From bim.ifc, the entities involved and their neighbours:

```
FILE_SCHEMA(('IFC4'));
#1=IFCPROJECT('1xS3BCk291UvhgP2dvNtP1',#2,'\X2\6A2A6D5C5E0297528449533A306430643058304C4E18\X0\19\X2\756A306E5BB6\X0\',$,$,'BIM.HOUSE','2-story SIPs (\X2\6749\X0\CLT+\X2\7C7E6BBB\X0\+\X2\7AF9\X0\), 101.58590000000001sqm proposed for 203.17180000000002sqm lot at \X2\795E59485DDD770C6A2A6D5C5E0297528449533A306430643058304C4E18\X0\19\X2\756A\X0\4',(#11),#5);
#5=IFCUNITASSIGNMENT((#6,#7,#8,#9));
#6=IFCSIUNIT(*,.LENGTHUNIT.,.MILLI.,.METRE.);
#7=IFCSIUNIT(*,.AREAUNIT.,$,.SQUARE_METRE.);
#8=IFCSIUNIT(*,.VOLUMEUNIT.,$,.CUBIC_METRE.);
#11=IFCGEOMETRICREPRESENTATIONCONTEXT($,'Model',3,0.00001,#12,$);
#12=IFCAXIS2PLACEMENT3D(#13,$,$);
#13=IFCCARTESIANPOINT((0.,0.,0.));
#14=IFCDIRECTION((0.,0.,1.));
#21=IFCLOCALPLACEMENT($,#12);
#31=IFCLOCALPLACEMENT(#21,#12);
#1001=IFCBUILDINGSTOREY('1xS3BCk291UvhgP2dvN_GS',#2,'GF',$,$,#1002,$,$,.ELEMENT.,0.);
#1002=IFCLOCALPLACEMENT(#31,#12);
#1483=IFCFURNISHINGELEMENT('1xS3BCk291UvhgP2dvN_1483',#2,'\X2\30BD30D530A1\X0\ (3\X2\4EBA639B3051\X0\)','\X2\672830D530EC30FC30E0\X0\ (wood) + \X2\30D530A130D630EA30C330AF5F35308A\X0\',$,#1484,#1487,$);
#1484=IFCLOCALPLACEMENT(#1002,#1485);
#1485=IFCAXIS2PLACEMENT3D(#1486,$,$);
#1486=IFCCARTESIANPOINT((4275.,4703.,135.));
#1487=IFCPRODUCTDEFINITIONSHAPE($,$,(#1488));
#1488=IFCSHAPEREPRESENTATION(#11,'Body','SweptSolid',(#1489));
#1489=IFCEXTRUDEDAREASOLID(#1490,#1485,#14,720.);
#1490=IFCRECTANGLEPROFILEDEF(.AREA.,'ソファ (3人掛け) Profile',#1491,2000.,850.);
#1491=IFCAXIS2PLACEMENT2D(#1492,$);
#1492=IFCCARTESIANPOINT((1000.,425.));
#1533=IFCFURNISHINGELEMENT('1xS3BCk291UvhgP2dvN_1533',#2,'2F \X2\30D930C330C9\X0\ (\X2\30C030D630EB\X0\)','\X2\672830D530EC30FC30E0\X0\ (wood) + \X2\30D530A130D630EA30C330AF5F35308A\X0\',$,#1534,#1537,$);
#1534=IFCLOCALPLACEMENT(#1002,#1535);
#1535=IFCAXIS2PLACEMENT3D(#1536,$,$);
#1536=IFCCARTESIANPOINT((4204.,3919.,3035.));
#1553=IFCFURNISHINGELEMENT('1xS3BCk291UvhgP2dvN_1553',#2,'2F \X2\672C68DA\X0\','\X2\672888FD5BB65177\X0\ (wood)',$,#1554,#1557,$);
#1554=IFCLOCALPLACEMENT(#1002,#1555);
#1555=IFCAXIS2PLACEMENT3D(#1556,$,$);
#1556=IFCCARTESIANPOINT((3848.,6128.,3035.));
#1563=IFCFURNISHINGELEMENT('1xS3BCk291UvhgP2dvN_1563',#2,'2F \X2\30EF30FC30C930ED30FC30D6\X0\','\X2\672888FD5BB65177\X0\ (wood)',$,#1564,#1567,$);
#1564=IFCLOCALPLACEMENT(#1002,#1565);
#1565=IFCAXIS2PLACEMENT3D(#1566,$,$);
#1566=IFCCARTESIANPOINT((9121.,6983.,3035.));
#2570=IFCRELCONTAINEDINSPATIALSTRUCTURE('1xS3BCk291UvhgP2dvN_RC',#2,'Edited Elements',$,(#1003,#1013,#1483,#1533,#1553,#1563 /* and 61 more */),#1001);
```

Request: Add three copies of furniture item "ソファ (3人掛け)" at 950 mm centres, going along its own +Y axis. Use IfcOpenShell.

```python
import ifcopenshell
import ifcopenshell.api.geometry
import ifcopenshell.api.root
import ifcopenshell.util.element
import ifcopenshell.util.placement
import ifcopenshell.util.unit

model = ifcopenshell.open("bim.ifc")
unit_scale = ifcopenshell.util.unit.calculate_unit_scale(model)


def reuse_history(source, copy):
    """copy_class also copies each property set's owner history, people and application; keep the originals."""
    for rel in copy.IsDefinedBy:
        if rel.is_a("IfcRelDefinesByProperties") and (history := rel.RelatingPropertyDefinition.OwnerHistory):
            rel.RelatingPropertyDefinition.OwnerHistory = source.OwnerHistory
            ifcopenshell.util.element.remove_deep2(model, history)


source = model.by_guid("1xS3BCk291UvhgP2dvN_1483")
base = ifcopenshell.util.placement.get_local_placement(source.ObjectPlacement)
step = base[:3, 1] * 0.95 / unit_scale

for i in range(1, 4):
    copy = ifcopenshell.api.root.copy_class(model, product=source)
    copy.Representation = ifcopenshell.util.element.copy_deep(
        model, source.Representation, exclude=["IfcGeometricRepresentationContext", "IfcRepresentationMap"]
    )
    reuse_history(source, copy)
    matrix = base.copy()
    matrix[:3, 3] += i * step
    print("added at", matrix[:3, 3].round(3) + 0.0)
    ifcopenshell.api.geometry.edit_object_placement(model, product=copy, matrix=matrix, is_si=False)

model.write("bim_v2.ifc")
```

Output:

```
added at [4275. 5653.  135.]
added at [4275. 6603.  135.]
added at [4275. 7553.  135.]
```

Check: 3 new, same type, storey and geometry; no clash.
